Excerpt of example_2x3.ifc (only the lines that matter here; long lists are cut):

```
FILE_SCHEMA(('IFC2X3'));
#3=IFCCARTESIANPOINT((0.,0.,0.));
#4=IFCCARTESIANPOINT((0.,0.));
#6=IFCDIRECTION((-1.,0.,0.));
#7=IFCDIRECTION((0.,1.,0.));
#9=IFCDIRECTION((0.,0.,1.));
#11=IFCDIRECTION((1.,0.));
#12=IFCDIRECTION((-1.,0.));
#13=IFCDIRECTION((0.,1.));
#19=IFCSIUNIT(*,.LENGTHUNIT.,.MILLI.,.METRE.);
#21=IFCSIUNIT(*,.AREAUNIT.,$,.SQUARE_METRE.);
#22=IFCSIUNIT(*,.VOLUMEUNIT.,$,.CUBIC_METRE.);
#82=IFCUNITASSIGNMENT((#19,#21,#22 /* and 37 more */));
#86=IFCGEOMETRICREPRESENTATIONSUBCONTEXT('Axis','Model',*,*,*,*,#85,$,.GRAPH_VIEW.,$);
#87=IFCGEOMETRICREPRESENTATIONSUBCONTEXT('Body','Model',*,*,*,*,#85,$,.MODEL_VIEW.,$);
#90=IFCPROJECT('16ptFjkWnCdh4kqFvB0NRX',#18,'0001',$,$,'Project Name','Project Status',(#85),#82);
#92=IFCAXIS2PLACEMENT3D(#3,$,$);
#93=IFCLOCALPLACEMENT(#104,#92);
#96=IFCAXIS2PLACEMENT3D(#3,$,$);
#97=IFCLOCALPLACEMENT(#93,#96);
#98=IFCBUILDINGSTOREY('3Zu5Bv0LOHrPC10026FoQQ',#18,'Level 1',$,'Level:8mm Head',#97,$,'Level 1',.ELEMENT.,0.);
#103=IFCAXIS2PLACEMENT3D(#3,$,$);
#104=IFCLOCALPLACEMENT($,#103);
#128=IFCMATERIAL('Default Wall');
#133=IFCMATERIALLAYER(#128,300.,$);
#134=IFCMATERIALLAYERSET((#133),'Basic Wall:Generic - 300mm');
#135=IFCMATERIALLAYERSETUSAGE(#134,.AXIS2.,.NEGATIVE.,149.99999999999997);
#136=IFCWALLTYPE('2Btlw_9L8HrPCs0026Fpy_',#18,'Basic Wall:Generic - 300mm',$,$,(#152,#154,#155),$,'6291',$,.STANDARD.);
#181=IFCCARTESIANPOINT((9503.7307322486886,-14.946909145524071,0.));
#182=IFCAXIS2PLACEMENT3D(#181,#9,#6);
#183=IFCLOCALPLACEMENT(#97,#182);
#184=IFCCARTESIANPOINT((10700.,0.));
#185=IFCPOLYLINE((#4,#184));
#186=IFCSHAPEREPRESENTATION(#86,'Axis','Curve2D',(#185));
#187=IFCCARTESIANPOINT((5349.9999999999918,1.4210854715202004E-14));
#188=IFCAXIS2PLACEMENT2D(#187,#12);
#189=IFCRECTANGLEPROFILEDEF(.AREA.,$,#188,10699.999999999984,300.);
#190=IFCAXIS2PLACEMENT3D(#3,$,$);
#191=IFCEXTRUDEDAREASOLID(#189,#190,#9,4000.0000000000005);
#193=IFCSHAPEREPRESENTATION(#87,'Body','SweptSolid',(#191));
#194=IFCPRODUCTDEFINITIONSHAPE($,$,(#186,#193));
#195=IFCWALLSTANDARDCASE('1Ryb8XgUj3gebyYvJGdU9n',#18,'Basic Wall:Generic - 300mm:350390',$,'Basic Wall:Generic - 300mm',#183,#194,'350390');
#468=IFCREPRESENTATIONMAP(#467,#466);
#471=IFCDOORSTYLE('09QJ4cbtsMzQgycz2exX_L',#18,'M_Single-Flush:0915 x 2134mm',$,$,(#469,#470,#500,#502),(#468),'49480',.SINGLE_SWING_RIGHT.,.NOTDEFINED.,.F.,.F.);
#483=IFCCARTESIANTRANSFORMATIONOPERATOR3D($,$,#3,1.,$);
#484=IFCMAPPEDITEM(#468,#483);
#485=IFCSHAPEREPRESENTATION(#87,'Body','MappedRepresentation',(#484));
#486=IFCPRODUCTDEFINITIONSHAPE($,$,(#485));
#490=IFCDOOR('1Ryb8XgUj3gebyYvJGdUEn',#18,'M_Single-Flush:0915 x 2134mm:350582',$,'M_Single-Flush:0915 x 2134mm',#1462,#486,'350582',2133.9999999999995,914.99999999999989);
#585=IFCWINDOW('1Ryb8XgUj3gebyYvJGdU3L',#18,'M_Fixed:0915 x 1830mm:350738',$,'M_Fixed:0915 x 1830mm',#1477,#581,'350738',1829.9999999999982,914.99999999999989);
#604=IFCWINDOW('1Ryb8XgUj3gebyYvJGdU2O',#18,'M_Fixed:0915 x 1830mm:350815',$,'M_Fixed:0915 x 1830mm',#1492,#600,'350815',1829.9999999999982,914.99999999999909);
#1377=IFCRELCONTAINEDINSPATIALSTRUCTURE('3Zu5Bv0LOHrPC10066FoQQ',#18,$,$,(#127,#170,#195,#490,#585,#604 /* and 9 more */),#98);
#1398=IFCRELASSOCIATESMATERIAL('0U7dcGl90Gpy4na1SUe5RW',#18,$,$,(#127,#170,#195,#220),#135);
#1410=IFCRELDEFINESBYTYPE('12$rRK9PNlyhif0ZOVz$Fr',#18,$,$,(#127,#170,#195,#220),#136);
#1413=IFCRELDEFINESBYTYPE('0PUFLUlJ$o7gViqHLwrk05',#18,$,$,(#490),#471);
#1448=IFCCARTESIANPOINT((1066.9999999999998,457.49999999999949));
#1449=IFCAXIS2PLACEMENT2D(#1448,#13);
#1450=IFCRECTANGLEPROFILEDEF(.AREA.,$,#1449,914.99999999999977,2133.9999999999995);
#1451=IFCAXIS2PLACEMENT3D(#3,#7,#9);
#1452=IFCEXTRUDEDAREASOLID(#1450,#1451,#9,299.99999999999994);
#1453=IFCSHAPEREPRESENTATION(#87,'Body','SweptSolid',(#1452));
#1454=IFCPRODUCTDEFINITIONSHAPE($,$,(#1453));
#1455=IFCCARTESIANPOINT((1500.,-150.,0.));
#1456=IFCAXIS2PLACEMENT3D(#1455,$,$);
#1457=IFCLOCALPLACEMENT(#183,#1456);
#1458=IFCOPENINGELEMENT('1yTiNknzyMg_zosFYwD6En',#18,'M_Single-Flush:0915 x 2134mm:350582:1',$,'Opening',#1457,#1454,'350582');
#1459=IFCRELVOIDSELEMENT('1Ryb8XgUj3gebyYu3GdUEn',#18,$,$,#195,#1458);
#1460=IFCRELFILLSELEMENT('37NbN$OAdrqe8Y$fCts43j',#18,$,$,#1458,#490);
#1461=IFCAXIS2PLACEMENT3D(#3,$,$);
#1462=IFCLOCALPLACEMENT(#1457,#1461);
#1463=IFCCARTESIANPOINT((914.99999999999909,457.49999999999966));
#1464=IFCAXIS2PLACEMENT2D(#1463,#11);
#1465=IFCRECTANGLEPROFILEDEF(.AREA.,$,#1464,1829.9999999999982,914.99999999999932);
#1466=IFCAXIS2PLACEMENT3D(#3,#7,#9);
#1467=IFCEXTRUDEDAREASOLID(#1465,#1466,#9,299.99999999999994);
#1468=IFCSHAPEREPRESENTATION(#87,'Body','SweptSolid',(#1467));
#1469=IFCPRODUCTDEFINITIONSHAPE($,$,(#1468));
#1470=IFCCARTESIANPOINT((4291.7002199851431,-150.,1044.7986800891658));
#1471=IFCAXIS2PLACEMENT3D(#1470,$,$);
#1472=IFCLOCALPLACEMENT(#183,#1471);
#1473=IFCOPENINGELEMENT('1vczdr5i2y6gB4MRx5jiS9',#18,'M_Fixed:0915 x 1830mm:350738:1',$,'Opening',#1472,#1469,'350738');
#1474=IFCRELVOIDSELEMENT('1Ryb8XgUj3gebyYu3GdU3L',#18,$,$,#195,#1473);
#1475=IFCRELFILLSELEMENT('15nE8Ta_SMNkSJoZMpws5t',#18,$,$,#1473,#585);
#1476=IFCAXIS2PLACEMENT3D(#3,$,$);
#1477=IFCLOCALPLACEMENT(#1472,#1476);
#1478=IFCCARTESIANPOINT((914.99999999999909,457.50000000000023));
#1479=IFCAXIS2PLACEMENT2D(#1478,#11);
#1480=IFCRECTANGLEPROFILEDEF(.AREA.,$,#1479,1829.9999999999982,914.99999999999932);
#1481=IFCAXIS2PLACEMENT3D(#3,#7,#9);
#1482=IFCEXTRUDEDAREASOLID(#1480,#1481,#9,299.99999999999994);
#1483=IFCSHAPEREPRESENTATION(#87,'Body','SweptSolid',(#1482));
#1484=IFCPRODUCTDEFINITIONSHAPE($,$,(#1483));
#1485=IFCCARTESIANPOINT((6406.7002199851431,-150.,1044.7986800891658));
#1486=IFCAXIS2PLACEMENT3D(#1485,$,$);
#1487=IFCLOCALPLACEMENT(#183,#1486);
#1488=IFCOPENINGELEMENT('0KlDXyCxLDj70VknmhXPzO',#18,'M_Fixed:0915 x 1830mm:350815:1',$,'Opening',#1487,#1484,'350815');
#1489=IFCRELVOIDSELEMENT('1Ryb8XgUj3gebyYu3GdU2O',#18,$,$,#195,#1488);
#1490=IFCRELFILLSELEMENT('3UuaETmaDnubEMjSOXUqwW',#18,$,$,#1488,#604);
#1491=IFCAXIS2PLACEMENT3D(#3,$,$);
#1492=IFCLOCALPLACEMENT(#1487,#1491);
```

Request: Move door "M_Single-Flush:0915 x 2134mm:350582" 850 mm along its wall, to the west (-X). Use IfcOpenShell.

```python
import ifcopenshell
import ifcopenshell.api.geometry
import ifcopenshell.util.placement

model = ifcopenshell.open("example_2x3.ifc")

door = model.by_guid("1Ryb8XgUj3gebyYvJGdUEn")
opening = door.FillsVoids[0].RelatingOpeningElement
wall = opening.VoidsElements[0].RelatingBuildingElement

wall_matrix = ifcopenshell.util.placement.get_local_placement(wall.ObjectPlacement)
shift = wall_matrix[:3, 0] * 850.0
before = ifcopenshell.util.placement.get_local_placement(door.ObjectPlacement)[:3, 3].copy()

# The door is placed relative to its opening, so it follows when the opening moves.
matrix = ifcopenshell.util.placement.get_local_placement(opening.ObjectPlacement)
matrix[:3, 3] += shift
ifcopenshell.api.geometry.edit_object_placement(
    model, product=opening, matrix=matrix, is_si=False, should_transform_children=True
)

after = ifcopenshell.util.placement.get_local_placement(door.ObjectPlacement)[:3, 3]
print("door moved by", (after - before).round(3) + 0.0)

model.write("example_2x3_v2.ifc")
```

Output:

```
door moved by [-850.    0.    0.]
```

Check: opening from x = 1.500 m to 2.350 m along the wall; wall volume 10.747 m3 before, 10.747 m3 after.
